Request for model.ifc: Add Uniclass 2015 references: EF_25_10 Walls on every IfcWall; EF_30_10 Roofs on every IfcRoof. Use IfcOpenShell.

First a look at what the model holds.

```python
import ifcopenshell

model = ifcopenshell.open("model.ifc")
print(model.schema)
print("classifications:", [c.Name for c in model.by_type("IfcClassification")])
for ifc_class in ("IfcDoor", "IfcRoof", "IfcStair", "IfcWall", "IfcWindow"):
    print(ifc_class, len(model.by_type(ifc_class)))
```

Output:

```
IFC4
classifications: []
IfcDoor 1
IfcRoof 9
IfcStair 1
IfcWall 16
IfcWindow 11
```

```python
import ifcopenshell
import ifcopenshell.api.classification

model = ifcopenshell.open("model.ifc")

system = ifcopenshell.api.classification.add_classification(model, classification="Uniclass 2015")

codes = {
    "IfcWall": ("EF_25_10", "Walls"),
    "IfcRoof": ("EF_30_10", "Roofs"),
}
for ifc_class, (code, name) in codes.items():
    products = model.by_type(ifc_class)
    ifcopenshell.api.classification.add_reference(
        model, products=products, classification=system, identification=code, name=name
    )
    print(code, len(products))

model.write("model-out.ifc")
```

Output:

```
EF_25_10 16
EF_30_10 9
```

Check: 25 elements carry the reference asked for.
